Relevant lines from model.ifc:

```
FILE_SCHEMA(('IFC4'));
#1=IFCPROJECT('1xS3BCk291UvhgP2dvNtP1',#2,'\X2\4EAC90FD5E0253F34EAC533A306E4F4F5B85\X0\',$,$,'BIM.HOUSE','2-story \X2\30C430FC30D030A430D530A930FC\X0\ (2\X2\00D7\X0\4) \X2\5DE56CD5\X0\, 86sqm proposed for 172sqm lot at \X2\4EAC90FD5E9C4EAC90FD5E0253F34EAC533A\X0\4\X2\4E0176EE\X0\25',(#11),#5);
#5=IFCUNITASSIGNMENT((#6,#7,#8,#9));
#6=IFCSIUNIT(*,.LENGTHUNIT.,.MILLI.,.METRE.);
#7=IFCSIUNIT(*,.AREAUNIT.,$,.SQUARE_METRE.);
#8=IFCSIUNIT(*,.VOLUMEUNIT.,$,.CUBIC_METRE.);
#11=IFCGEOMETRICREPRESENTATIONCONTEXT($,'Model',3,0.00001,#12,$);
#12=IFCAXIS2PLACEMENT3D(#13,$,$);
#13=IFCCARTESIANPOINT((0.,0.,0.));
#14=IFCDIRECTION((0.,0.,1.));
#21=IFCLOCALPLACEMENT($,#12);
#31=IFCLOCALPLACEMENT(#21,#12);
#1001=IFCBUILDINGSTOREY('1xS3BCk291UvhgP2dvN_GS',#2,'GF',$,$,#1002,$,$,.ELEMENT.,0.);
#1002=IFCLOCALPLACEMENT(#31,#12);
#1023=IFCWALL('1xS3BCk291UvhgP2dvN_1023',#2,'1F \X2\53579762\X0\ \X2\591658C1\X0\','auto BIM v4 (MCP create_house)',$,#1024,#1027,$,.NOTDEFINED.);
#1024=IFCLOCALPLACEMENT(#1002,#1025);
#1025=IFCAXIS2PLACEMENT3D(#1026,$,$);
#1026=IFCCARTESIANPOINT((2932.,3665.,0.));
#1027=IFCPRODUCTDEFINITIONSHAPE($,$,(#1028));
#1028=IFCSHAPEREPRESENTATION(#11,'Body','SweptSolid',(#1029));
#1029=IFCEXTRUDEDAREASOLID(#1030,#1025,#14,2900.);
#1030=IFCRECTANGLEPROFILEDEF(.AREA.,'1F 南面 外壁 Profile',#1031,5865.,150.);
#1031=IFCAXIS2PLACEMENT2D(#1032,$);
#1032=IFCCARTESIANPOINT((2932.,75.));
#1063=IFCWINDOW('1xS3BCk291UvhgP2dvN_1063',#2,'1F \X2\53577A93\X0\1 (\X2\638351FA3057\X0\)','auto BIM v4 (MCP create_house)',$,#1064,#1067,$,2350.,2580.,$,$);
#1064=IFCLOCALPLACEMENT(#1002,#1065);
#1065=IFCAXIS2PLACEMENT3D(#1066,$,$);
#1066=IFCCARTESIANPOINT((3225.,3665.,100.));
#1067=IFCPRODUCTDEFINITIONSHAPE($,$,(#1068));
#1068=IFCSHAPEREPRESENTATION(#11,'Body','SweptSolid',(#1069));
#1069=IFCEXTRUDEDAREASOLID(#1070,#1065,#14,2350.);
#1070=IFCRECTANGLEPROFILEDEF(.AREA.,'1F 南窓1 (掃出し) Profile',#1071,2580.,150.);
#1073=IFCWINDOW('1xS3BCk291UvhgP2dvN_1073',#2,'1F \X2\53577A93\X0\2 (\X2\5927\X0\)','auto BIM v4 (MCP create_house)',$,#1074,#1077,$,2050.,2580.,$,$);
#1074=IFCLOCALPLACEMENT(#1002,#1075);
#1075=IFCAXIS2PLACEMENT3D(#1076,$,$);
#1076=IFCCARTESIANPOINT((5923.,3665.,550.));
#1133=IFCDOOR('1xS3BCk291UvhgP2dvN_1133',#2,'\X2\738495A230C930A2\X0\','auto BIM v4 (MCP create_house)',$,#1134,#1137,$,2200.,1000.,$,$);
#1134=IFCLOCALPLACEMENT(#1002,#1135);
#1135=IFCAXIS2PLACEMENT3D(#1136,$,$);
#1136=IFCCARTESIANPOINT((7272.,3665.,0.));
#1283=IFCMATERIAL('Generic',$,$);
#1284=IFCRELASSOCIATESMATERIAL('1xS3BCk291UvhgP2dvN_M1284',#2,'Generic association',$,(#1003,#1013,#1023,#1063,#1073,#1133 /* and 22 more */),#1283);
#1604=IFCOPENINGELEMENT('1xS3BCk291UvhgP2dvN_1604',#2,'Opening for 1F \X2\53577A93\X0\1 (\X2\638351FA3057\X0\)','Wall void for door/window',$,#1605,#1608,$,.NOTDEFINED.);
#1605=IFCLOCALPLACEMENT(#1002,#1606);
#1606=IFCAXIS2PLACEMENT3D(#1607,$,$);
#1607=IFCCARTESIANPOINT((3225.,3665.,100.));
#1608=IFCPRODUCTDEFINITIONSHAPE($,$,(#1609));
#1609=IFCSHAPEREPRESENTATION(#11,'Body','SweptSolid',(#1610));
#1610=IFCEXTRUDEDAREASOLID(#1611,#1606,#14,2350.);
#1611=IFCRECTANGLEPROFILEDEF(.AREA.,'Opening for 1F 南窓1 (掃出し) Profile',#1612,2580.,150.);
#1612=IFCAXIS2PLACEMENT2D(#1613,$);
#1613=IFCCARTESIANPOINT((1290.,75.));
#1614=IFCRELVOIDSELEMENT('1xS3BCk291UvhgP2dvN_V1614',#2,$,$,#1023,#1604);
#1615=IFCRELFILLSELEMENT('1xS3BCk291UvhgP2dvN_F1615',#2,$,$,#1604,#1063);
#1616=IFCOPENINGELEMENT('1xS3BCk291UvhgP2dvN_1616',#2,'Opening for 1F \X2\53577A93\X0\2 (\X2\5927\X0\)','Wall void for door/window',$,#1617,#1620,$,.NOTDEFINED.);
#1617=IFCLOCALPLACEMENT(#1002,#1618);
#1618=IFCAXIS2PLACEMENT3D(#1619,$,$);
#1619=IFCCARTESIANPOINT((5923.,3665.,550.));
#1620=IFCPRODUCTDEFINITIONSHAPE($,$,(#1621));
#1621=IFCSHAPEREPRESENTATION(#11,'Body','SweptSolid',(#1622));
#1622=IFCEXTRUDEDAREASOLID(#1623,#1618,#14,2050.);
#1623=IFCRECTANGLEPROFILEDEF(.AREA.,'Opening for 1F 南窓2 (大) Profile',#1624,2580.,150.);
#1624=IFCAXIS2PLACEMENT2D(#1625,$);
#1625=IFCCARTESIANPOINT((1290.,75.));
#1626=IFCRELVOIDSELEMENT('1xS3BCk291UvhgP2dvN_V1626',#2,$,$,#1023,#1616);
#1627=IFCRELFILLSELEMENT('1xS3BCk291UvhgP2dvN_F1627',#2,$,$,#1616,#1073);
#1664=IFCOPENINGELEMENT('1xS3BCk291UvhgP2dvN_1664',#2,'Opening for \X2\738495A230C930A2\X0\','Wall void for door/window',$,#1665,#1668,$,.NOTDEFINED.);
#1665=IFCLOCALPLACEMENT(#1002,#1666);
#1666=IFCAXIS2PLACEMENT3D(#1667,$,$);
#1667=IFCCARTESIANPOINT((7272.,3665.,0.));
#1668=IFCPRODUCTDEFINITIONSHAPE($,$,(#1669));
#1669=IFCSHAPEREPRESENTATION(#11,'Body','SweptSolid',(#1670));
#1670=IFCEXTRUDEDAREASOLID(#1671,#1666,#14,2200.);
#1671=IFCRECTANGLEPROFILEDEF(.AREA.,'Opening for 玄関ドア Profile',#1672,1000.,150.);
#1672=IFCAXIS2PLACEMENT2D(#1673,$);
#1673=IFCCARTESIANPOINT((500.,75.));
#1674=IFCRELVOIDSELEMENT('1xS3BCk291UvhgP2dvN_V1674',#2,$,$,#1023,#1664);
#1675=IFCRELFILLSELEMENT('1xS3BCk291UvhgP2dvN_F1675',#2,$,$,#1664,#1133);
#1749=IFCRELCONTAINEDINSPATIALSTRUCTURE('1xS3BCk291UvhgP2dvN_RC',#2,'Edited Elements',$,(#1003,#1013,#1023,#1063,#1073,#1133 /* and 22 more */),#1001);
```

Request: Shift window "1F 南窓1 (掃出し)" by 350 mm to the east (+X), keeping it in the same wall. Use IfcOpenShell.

```python
import ifcopenshell
import ifcopenshell.api.geometry
import ifcopenshell.util.placement
import ifcopenshell.util.unit

model = ifcopenshell.open("model.ifc")
unit_scale = ifcopenshell.util.unit.calculate_unit_scale(model)

window = model.by_guid("1xS3BCk291UvhgP2dvN_1063")
opening = window.FillsVoids[0].RelatingOpeningElement
wall = opening.VoidsElements[0].RelatingBuildingElement

wall_matrix = ifcopenshell.util.placement.get_local_placement(wall.ObjectPlacement)
shift = wall_matrix[:3, 0] * 0.35 / unit_scale
before = ifcopenshell.util.placement.get_local_placement(window.ObjectPlacement)[:3, 3].copy()

# The window is not placed relative to its opening, so move both.
for product in (opening, window):
    matrix = ifcopenshell.util.placement.get_local_placement(product.ObjectPlacement)
    matrix[:3, 3] += shift
    ifcopenshell.api.geometry.edit_object_placement(model, product=product, matrix=matrix, is_si=False)

after = ifcopenshell.util.placement.get_local_placement(window.ObjectPlacement)[:3, 3]
print("window moved by", (after - before).round(3) + 0.0)

model.write("model_edited.ifc")
```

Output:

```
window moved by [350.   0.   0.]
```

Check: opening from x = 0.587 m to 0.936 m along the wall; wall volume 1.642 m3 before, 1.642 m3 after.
